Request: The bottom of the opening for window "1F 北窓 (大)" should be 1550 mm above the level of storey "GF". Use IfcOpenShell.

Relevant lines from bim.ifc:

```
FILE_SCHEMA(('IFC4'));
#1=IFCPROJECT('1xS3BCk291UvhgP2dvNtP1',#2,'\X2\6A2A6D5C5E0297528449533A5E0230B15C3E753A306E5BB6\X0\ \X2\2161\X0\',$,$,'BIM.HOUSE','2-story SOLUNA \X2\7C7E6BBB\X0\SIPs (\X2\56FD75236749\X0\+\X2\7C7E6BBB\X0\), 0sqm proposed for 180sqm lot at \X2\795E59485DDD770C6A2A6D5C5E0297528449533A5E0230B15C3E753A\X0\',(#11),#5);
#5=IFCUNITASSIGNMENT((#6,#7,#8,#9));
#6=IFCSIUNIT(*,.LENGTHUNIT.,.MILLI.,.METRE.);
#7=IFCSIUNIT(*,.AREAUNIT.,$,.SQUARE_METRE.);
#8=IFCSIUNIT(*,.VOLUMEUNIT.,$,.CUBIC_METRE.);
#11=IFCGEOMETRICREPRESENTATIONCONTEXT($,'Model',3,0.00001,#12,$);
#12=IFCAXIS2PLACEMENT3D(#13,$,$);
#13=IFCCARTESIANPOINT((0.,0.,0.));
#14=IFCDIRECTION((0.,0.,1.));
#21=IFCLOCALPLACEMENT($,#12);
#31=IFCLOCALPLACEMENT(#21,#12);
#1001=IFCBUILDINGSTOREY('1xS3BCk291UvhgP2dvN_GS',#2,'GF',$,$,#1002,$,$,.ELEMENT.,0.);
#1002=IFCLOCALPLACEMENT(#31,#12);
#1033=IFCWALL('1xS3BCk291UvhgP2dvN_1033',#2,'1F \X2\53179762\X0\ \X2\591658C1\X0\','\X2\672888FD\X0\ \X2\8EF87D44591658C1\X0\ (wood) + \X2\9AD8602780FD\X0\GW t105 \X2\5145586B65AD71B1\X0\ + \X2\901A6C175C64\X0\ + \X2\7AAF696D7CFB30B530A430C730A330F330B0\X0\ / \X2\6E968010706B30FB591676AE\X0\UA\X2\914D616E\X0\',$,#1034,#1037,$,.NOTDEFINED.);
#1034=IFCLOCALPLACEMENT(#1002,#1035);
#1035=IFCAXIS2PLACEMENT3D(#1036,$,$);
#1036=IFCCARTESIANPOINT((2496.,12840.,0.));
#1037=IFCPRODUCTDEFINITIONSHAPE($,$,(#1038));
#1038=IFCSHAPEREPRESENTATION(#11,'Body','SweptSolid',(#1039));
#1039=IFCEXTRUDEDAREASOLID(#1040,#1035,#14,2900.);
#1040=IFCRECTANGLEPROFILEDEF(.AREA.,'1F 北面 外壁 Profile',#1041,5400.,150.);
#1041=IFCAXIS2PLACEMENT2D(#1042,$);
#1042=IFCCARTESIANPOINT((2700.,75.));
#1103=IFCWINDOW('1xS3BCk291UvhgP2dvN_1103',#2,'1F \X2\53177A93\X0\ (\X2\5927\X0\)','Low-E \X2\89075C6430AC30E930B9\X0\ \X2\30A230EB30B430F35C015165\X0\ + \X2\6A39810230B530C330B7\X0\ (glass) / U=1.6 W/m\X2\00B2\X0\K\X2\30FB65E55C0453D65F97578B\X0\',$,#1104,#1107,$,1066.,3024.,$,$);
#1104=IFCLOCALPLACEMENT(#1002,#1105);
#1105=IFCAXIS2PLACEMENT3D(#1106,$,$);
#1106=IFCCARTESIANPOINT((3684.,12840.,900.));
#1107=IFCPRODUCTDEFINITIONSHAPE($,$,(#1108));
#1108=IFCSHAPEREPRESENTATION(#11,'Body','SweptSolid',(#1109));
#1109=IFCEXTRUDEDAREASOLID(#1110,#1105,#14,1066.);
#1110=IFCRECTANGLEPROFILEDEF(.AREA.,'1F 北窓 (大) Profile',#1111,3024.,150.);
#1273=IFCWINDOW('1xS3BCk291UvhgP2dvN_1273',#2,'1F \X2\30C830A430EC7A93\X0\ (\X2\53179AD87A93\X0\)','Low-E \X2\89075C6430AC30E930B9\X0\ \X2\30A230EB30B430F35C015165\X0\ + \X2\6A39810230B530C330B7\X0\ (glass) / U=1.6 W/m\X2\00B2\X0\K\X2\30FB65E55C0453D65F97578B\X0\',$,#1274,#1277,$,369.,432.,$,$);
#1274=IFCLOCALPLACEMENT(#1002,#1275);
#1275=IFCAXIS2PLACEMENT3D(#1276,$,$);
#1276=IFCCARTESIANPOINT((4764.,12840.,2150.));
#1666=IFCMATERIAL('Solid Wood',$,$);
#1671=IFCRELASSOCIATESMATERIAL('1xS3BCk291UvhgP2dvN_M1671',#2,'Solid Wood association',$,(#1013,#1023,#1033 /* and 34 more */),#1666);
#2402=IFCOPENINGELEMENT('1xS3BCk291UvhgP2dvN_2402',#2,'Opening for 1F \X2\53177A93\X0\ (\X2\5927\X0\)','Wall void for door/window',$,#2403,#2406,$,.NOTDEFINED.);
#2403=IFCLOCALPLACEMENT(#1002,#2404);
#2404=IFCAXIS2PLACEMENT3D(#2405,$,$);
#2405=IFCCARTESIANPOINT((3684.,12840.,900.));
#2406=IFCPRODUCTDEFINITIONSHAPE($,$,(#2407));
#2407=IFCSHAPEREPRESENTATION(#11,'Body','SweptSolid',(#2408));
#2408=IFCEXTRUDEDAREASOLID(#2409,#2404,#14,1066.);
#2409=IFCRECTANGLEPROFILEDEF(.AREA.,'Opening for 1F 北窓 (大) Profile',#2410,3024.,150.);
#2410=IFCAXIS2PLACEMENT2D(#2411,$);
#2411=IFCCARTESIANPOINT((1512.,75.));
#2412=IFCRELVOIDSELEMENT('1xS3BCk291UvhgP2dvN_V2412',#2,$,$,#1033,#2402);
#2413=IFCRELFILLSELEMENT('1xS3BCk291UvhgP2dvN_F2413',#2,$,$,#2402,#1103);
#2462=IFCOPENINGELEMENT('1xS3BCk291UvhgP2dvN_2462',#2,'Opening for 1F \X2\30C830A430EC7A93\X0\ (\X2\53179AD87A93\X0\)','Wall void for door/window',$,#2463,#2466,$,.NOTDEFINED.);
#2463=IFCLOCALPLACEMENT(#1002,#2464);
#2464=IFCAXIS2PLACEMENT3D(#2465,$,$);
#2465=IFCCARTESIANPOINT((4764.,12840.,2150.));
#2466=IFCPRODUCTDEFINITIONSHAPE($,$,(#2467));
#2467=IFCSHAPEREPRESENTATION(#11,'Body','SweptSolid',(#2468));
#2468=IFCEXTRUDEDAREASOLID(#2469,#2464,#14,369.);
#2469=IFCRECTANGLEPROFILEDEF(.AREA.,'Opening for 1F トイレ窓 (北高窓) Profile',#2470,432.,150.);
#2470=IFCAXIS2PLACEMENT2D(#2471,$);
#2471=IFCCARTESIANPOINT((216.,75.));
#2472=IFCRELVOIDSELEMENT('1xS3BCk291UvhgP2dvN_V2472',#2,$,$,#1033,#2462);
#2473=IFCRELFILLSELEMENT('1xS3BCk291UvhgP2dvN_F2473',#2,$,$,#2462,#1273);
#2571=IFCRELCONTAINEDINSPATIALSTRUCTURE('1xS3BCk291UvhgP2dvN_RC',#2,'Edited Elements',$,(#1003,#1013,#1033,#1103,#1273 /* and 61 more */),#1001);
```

```python
import numpy as np
import ifcopenshell
import ifcopenshell.api.geometry
import ifcopenshell.geom
import ifcopenshell.util.element
import ifcopenshell.util.placement
import ifcopenshell.util.shape
import ifcopenshell.util.unit

model = ifcopenshell.open("bim.ifc")
unit_scale = ifcopenshell.util.unit.calculate_unit_scale(model)

window = model.by_guid("1xS3BCk291UvhgP2dvN_1103")
opening = window.FillsVoids[0].RelatingOpeningElement
storey = ifcopenshell.util.element.get_container(window, ifc_class="IfcBuildingStorey")
level = ifcopenshell.util.placement.get_local_placement(storey.ObjectPlacement)[2, 3]

# The opening's origin need not be at the sill, so measure its lowest point.
shape = ifcopenshell.geom.create_shape(ifcopenshell.geom.settings(), opening)
bottom = ifcopenshell.util.shape.get_shape_bottom_elevation(shape, shape.geometry) / unit_scale
dz = level + 1.55 / unit_scale - bottom

shift = np.array([0.0, 0.0, dz])
# The window is not placed relative to its opening, so move both.
for product in (opening, window):
    matrix = ifcopenshell.util.placement.get_local_placement(product.ObjectPlacement)
    matrix[:3, 3] += shift
    ifcopenshell.api.geometry.edit_object_placement(model, product=product, matrix=matrix, is_si=False)

print(f"moved by {dz * unit_scale:+.3f} m")

model.write("bim_v2.ifc")
```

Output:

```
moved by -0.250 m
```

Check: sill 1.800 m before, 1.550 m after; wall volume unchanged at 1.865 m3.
